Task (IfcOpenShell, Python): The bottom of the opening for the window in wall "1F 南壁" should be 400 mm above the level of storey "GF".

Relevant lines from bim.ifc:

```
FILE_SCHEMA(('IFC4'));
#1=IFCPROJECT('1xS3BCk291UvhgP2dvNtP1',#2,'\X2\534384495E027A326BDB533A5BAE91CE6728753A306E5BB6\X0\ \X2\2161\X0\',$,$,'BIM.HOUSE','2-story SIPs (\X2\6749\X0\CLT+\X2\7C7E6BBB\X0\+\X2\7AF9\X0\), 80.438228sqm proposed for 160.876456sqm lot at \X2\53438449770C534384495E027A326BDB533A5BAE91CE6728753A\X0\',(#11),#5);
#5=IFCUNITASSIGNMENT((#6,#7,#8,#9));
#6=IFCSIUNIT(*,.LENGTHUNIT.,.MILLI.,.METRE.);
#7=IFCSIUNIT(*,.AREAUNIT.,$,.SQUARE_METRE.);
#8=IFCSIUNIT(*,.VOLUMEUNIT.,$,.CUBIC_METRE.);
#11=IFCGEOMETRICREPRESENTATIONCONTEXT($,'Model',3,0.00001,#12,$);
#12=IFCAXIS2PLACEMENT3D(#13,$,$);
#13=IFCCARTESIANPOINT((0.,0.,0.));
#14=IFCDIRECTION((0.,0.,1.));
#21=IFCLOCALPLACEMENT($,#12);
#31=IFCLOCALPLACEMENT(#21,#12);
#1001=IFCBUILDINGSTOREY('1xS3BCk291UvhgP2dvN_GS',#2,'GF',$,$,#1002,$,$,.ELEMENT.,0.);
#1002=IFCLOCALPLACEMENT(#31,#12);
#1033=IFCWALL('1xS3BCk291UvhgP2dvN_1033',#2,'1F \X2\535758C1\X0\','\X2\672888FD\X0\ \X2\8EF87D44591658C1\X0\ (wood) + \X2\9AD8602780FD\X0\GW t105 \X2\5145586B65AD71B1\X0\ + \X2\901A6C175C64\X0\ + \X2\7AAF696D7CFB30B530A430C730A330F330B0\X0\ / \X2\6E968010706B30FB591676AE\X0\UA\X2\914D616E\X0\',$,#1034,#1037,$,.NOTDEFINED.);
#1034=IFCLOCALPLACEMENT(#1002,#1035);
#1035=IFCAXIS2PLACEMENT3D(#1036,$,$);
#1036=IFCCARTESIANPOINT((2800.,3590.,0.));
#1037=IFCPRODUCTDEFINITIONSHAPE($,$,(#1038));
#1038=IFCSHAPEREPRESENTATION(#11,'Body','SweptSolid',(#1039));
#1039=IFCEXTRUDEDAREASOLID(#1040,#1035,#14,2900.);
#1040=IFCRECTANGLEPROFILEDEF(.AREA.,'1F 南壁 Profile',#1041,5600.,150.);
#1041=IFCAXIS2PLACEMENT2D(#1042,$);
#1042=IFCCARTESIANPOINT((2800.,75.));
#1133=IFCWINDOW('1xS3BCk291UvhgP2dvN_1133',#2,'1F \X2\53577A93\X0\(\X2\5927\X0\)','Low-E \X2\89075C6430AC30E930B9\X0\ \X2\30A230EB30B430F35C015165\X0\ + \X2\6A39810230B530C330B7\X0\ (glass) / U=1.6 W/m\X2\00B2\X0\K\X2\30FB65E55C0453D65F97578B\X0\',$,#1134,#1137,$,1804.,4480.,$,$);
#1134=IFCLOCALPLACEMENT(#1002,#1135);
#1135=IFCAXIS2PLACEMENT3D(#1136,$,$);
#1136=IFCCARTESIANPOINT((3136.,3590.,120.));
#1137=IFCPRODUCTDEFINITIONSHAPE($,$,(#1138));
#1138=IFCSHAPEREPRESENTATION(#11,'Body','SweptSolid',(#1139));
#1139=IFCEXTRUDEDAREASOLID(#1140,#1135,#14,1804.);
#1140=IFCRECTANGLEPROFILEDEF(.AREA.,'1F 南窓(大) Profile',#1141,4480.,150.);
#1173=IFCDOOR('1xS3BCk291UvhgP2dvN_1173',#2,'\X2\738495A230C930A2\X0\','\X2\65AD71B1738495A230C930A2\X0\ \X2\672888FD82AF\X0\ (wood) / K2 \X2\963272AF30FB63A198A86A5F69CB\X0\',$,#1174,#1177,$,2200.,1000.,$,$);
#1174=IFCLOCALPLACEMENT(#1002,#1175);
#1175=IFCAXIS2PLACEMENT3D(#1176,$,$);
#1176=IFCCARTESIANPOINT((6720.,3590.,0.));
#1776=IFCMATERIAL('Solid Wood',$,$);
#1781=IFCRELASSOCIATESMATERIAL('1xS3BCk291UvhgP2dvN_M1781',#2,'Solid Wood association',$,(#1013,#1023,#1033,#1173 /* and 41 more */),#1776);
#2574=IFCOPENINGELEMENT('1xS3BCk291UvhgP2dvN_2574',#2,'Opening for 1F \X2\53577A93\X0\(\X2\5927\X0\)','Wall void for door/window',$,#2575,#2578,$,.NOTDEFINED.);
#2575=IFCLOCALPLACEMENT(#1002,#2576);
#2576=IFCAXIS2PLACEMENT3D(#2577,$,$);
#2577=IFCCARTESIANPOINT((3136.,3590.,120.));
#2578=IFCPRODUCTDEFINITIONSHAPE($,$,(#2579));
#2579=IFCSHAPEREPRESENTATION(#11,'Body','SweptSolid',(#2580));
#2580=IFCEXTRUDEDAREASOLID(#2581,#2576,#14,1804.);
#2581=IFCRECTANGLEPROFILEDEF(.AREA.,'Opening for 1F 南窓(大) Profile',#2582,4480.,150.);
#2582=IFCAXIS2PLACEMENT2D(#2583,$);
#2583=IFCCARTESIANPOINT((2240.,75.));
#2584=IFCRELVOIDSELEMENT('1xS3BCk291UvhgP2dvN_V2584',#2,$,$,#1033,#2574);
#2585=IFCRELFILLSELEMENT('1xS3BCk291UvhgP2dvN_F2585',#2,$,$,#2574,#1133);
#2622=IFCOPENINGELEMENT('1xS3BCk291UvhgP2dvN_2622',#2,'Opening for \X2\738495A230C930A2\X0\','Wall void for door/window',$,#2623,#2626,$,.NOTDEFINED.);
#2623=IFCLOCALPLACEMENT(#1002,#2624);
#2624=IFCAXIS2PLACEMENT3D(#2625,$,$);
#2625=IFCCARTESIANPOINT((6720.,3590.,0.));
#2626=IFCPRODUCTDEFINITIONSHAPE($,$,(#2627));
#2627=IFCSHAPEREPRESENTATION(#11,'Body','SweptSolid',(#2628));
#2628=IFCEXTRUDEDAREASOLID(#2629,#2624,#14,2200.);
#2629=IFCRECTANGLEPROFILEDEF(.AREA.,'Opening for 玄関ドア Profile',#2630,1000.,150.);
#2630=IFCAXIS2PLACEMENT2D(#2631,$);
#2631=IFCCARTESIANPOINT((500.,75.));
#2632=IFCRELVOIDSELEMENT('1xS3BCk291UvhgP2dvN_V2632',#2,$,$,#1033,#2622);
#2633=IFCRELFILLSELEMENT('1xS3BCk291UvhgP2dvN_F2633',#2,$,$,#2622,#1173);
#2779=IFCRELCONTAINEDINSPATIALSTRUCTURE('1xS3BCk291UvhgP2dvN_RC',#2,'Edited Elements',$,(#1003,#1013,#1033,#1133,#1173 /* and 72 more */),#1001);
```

```python
import numpy as np
import ifcopenshell
import ifcopenshell.api.geometry
import ifcopenshell.geom
import ifcopenshell.util.element
import ifcopenshell.util.placement
import ifcopenshell.util.shape
import ifcopenshell.util.unit

model = ifcopenshell.open("bim.ifc")
unit_scale = ifcopenshell.util.unit.calculate_unit_scale(model)

window = model.by_guid("1xS3BCk291UvhgP2dvN_1133")
opening = window.FillsVoids[0].RelatingOpeningElement
storey = ifcopenshell.util.element.get_container(window, ifc_class="IfcBuildingStorey")
level = ifcopenshell.util.placement.get_local_placement(storey.ObjectPlacement)[2, 3]

# The opening's origin need not be at the sill, so measure its lowest point.
shape = ifcopenshell.geom.create_shape(ifcopenshell.geom.settings(), opening)
bottom = ifcopenshell.util.shape.get_shape_bottom_elevation(shape, shape.geometry) / unit_scale
dz = level + 0.4 / unit_scale - bottom

shift = np.array([0.0, 0.0, dz])
# The window is not placed relative to its opening, so move both.
for product in (opening, window):
    matrix = ifcopenshell.util.placement.get_local_placement(product.ObjectPlacement)
    matrix[:3, 3] += shift
    ifcopenshell.api.geometry.edit_object_placement(model, product=product, matrix=matrix, is_si=False)

print(f"moved by {dz * unit_scale:+.3f} m")

model.write("bim_v2.ifc")
```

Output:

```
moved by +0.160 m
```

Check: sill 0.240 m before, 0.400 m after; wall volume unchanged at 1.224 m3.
